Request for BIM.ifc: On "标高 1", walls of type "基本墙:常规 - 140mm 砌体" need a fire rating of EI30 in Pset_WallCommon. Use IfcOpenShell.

First a look at what the model holds.

```python
import ifcopenshell
import ifcopenshell.util.element

model = ifcopenshell.open("BIM.ifc")
print(model.schema)
storey = next(s for s in model.by_type("IfcBuildingStorey") if s.Name == "标高 1")
walls = [e for e in ifcopenshell.util.element.get_decomposition(storey) if e.is_a("IfcWall")]
seen = {}
for e in walls:
    element_type = ifcopenshell.util.element.get_type(e)
    key = (element_type.Name if element_type != e and element_type else None, ifcopenshell.util.element.get_pset(e, "Pset_WallCommon", "FireRating"))
    seen[key] = seen.get(key, 0) + 1
for (name, value), count in sorted(seen.items(), key=str):
    print(count, "x", name, "|", value)
```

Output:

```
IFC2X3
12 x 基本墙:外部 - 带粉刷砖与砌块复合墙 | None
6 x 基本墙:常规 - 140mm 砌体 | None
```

```python
import ifcopenshell
import ifcopenshell.api.pset
import ifcopenshell.util.element

model = ifcopenshell.open("BIM.ifc")

storey = next(s for s in model.by_type("IfcBuildingStorey") if s.Name == "标高 1")
walls = [e for e in ifcopenshell.util.element.get_decomposition(storey) if e.is_a("IfcWall")]

count = 0
for e in walls:
    element_type = ifcopenshell.util.element.get_type(e)
    if element_type in (None, e) or element_type.Name != "基本墙:常规 - 140mm 砌体":
        continue
    # add_pset returns the element's existing set when there is one.
    pset = ifcopenshell.api.pset.add_pset(model, product=e, name="Pset_WallCommon")
    ifcopenshell.api.pset.edit_pset(model, pset=pset, properties={"FireRating": "EI30"})
    count += 1

print(count, "walls updated")

model.write("BIM_updated.ifc")
```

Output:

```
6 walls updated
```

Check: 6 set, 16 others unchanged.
